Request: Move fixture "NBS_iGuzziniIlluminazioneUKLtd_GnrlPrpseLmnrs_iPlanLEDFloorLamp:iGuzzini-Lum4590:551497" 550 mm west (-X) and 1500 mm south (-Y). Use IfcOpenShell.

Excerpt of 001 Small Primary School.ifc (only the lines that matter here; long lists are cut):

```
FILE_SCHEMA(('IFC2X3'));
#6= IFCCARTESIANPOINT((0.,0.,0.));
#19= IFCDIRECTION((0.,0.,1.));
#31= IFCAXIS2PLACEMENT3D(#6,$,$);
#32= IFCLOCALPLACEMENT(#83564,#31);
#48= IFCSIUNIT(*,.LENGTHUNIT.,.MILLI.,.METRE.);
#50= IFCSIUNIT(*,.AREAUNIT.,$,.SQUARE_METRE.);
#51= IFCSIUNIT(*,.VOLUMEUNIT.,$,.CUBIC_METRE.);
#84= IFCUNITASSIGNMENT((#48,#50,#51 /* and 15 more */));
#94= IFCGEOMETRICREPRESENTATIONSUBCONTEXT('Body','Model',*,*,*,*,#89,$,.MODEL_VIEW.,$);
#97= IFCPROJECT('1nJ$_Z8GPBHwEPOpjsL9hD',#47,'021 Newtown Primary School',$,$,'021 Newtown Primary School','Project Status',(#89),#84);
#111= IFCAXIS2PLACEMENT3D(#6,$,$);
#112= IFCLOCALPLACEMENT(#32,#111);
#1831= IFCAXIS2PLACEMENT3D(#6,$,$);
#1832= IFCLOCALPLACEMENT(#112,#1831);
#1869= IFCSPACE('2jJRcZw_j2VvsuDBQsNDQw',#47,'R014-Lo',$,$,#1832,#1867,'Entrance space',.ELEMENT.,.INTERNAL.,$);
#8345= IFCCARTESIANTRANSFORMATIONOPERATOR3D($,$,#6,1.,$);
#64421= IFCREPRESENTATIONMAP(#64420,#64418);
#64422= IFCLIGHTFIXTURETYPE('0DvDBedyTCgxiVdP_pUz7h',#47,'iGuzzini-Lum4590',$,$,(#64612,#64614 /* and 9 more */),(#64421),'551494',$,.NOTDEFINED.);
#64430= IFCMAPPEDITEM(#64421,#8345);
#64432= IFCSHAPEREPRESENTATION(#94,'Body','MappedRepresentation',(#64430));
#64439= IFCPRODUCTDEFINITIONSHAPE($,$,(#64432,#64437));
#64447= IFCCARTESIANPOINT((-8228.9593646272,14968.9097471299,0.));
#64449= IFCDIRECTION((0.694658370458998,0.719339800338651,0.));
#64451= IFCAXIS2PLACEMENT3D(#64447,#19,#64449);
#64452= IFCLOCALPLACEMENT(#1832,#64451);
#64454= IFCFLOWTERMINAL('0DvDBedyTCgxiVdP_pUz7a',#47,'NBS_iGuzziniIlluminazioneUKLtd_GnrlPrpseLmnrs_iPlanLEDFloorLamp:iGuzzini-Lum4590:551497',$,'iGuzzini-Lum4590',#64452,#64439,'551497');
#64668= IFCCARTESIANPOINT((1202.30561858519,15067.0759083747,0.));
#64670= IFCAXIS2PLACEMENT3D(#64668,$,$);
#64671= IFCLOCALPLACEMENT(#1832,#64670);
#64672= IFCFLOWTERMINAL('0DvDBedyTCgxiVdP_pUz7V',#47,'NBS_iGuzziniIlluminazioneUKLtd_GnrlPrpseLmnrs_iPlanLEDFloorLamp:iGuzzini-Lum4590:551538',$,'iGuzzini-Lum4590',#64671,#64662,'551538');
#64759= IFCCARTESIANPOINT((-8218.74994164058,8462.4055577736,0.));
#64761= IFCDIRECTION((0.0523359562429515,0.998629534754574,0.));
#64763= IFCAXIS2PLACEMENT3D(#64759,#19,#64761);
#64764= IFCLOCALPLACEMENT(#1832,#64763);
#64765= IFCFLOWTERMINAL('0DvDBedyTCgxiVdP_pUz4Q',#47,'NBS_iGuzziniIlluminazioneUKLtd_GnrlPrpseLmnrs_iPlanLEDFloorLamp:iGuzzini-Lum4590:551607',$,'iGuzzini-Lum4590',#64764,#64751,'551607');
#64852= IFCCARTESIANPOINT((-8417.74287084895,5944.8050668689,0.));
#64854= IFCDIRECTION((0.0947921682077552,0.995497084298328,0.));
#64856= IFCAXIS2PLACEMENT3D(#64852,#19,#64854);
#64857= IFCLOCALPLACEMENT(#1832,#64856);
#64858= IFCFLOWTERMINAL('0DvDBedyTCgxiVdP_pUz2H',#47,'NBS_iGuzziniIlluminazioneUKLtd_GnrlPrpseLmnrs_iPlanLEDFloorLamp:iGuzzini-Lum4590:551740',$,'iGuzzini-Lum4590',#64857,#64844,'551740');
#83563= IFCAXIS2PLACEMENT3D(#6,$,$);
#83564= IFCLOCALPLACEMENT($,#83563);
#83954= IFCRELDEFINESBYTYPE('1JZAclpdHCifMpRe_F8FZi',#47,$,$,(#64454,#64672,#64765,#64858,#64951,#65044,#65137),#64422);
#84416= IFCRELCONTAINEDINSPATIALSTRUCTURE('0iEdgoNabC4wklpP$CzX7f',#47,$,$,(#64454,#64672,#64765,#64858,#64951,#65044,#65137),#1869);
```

```python
import ifcopenshell
import ifcopenshell.api.geometry
import ifcopenshell.util.placement

model = ifcopenshell.open("001 Small Primary School.ifc")

item = model.by_guid("0DvDBedyTCgxiVdP_pUz7a")
matrix = ifcopenshell.util.placement.get_local_placement(item.ObjectPlacement)
matrix[0, 3] -= 550.0
matrix[1, 3] -= 1500.0
ifcopenshell.api.geometry.edit_object_placement(model, product=item, matrix=matrix, is_si=False)

print(ifcopenshell.util.placement.get_local_placement(item.ObjectPlacement).round(3) + 0.0)

model.write("001 Small Primary School-out.ifc")
```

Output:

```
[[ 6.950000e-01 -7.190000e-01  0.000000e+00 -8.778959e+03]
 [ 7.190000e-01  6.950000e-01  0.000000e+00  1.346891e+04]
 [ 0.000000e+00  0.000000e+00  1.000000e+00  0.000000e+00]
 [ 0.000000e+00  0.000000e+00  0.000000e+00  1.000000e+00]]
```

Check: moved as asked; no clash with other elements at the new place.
